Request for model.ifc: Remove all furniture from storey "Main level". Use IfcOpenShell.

First a look at what the model holds.

```python
import ifcopenshell
import ifcopenshell.util.element

model = ifcopenshell.open("model.ifc")
print(model.schema)
storey = next(s for s in model.by_type("IfcBuildingStorey") if s.Name == "Main level")
furniture = [e for e in ifcopenshell.util.element.get_decomposition(storey) if e.is_a("IfcFurnishingElement")]
seen = {}
for e in furniture:
    element_type = ifcopenshell.util.element.get_type(e)
    name = element_type.Name if element_type not in (None, e) else None
    seen[name] = seen.get(name, 0) + 1
for name, count in sorted(seen.items(), key=str):
    print(count, "x", name)
```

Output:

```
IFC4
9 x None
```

```python
import ifcopenshell
import ifcopenshell.api.root
import ifcopenshell.util.element

model = ifcopenshell.open("model.ifc")

storey = next(s for s in model.by_type("IfcBuildingStorey") if s.Name == "Main level")
furniture = [e for e in ifcopenshell.util.element.get_decomposition(storey) if e.is_a("IfcFurnishingElement")]

for e in furniture:
    ifcopenshell.api.root.remove_product(model, product=e)
print(len(furniture), "removed")

model.write("model_v2.ifc")
```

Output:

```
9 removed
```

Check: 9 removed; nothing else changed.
